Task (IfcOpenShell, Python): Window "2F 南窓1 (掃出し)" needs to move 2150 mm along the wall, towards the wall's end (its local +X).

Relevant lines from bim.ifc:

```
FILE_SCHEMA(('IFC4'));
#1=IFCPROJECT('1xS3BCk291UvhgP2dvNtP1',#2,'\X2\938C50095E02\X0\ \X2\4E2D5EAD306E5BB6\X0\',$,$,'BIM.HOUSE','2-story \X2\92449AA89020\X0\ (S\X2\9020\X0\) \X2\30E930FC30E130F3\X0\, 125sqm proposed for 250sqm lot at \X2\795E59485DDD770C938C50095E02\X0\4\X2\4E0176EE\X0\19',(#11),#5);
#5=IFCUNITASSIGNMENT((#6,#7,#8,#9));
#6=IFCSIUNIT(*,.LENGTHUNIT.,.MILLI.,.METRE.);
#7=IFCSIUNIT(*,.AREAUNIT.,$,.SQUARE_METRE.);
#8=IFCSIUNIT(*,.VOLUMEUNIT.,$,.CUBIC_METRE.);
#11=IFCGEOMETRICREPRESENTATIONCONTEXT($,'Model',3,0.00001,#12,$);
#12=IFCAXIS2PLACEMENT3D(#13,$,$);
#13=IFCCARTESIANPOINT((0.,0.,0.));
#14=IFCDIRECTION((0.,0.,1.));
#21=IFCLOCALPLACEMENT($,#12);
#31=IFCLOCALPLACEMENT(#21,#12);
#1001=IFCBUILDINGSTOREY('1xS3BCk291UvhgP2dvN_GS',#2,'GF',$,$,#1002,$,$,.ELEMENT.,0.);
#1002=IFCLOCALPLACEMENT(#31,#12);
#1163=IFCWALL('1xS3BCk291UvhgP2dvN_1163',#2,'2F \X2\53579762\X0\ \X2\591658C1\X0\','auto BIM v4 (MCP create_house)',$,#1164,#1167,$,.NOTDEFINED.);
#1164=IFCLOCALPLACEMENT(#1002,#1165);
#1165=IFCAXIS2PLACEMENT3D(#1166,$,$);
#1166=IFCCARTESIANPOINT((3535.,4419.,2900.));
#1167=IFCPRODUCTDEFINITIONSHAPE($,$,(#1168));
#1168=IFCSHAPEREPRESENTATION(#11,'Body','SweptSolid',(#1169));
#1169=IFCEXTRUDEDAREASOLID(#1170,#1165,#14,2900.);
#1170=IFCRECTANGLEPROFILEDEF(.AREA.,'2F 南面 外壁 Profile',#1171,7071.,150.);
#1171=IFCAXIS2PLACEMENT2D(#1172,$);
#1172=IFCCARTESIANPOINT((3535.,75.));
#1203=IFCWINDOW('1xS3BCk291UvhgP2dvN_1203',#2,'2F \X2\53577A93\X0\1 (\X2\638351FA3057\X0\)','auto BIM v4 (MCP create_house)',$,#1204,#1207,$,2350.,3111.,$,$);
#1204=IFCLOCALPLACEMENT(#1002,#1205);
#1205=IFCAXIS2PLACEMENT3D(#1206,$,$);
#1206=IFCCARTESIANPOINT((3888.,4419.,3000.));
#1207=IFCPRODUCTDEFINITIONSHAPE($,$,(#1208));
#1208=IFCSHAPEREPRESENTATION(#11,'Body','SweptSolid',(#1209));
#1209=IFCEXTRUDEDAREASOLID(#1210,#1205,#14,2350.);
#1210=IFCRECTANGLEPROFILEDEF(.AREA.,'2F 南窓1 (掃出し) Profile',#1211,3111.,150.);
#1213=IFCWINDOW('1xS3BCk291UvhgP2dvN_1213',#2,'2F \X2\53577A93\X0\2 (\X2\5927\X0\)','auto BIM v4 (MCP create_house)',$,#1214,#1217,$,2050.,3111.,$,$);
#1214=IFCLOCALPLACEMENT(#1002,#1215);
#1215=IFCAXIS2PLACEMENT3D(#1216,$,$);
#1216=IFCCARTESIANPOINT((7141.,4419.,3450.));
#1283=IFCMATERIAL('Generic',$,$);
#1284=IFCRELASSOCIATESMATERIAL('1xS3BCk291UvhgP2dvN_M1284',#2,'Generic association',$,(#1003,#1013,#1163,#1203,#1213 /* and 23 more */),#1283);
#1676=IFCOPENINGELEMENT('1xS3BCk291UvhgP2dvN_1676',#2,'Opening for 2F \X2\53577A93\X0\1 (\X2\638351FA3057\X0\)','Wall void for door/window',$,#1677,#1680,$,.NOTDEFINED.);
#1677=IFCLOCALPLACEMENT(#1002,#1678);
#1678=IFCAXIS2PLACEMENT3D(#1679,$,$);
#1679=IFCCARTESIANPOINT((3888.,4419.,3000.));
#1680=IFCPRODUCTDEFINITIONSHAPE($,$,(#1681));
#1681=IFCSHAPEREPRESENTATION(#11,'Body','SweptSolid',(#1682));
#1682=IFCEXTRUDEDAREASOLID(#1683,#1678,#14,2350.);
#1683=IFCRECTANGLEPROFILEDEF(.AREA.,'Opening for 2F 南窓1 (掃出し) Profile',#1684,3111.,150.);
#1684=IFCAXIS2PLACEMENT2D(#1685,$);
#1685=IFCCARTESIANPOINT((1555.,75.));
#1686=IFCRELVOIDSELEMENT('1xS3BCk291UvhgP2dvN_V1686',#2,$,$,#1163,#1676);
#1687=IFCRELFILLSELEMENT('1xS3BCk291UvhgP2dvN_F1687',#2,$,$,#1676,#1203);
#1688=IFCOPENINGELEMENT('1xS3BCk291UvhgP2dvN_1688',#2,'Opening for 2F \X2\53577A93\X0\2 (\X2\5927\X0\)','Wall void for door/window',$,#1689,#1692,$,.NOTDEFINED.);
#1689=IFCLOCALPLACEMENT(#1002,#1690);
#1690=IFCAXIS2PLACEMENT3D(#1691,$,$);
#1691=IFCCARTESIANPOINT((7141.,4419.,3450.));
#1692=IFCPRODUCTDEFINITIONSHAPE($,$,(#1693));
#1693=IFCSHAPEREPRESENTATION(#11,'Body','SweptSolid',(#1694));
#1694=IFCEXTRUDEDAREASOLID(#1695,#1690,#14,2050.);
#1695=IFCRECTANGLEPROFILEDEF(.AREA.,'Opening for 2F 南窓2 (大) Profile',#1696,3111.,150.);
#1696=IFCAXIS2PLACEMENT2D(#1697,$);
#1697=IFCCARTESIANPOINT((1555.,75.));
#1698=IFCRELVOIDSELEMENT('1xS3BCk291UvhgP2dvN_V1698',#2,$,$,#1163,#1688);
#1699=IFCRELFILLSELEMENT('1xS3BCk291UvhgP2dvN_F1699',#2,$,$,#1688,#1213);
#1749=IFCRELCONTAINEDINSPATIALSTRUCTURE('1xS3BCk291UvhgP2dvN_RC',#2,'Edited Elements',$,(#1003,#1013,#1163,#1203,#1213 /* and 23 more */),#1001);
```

```python
import ifcopenshell
import ifcopenshell.api.geometry
import ifcopenshell.util.placement

model = ifcopenshell.open("bim.ifc")

window = model.by_guid("1xS3BCk291UvhgP2dvN_1203")
opening = window.FillsVoids[0].RelatingOpeningElement
wall = opening.VoidsElements[0].RelatingBuildingElement

wall_matrix = ifcopenshell.util.placement.get_local_placement(wall.ObjectPlacement)
shift = wall_matrix[:3, 0] * 2150.0
before = ifcopenshell.util.placement.get_local_placement(window.ObjectPlacement)[:3, 3].copy()

# The window is not placed relative to its opening, so move both.
for product in (opening, window):
    matrix = ifcopenshell.util.placement.get_local_placement(product.ObjectPlacement)
    matrix[:3, 3] += shift
    ifcopenshell.api.geometry.edit_object_placement(model, product=product, matrix=matrix, is_si=False)

after = ifcopenshell.util.placement.get_local_placement(window.ObjectPlacement)[:3, 3]
print("window moved by", (after - before).round(3) + 0.0)

model.write("bim-out.ifc")
```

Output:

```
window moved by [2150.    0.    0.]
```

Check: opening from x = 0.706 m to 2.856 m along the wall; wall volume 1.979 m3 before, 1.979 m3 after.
